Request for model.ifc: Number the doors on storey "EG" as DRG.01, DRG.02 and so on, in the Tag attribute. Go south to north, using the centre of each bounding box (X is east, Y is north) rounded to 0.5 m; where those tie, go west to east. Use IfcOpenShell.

First a look at what the model holds.

```python
import ifcopenshell
import ifcopenshell.util.element
import ifcopenshell.util.placement

model = ifcopenshell.open("model.ifc")
print(model.schema)
storey = next(s for s in model.by_type("IfcBuildingStorey") if s.Name == "EG")
doors = [e for e in ifcopenshell.util.element.get_decomposition(storey) if e.is_a("IfcDoor")]
for e in sorted(doors, key=lambda e: e.id()):
    origin = ifcopenshell.util.placement.get_local_placement(e.ObjectPlacement)[:3, 3]
    print(e.id(), e.Tag, e.Name, origin.round(2) + 0.0, sep=" | ")
```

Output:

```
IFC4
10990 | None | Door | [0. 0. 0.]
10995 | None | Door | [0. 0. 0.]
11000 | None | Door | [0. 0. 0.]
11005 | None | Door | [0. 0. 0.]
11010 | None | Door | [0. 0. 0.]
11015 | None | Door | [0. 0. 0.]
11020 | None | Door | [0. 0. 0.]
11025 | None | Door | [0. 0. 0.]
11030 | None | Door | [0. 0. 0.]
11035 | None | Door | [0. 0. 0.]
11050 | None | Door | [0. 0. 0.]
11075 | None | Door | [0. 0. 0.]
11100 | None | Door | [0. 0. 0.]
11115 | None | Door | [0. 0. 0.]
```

```python
import ifcopenshell
import ifcopenshell.geom
import ifcopenshell.util.element
import ifcopenshell.util.shape

model = ifcopenshell.open("model.ifc")
settings = ifcopenshell.geom.settings()
settings.set("use-world-coords", True)


def centre(element):
    shape = ifcopenshell.geom.create_shape(settings, element)
    return ifcopenshell.util.shape.get_bbox_centroid(shape.geometry)


storey = next(s for s in model.by_type("IfcBuildingStorey") if s.Name == "EG")
doors = [e for e in ifcopenshell.util.element.get_decomposition(storey) if e.is_a("IfcDoor")]

# Insertion points can sit at a corner or the storey origin, so sort by the geometry (in metres).
centres = {e: centre(e) for e in doors}
doors.sort(key=lambda e: (round(centres[e][1] / 0.5), centres[e][0]))

for i, e in enumerate(doors, start=1):
    number = f"DRG.{i:02d}"
    e.Tag = number
    print(e.id(), number)

model.write("model_v2.ifc")
```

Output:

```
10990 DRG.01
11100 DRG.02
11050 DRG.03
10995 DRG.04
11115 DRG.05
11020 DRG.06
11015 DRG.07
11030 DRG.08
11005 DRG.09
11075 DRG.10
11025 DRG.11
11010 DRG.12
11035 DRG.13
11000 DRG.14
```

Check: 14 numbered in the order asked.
